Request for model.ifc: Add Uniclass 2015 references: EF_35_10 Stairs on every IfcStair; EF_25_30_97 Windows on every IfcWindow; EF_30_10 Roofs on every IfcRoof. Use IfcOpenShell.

First a look at what the model holds.

```python
import ifcopenshell

model = ifcopenshell.open("model.ifc")
print(model.schema)
print("classifications:", [c.Name for c in model.by_type("IfcClassification")])
for ifc_class in ("IfcDoor", "IfcRoof", "IfcStair", "IfcWall", "IfcWindow"):
    print(ifc_class, len(model.by_type(ifc_class)))
```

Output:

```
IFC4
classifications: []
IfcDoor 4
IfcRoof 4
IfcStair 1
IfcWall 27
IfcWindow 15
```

```python
import ifcopenshell
import ifcopenshell.api.classification

model = ifcopenshell.open("model.ifc")

system = ifcopenshell.api.classification.add_classification(model, classification="Uniclass 2015")

codes = {
    "IfcStair": ("EF_35_10", "Stairs"),
    "IfcWindow": ("EF_25_30_97", "Windows"),
    "IfcRoof": ("EF_30_10", "Roofs"),
}
for ifc_class, (code, name) in codes.items():
    products = model.by_type(ifc_class)
    ifcopenshell.api.classification.add_reference(
        model, products=products, classification=system, identification=code, name=name
    )
    print(code, len(products))

model.write("model_edited.ifc")
```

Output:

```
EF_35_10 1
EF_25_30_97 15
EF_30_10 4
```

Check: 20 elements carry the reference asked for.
